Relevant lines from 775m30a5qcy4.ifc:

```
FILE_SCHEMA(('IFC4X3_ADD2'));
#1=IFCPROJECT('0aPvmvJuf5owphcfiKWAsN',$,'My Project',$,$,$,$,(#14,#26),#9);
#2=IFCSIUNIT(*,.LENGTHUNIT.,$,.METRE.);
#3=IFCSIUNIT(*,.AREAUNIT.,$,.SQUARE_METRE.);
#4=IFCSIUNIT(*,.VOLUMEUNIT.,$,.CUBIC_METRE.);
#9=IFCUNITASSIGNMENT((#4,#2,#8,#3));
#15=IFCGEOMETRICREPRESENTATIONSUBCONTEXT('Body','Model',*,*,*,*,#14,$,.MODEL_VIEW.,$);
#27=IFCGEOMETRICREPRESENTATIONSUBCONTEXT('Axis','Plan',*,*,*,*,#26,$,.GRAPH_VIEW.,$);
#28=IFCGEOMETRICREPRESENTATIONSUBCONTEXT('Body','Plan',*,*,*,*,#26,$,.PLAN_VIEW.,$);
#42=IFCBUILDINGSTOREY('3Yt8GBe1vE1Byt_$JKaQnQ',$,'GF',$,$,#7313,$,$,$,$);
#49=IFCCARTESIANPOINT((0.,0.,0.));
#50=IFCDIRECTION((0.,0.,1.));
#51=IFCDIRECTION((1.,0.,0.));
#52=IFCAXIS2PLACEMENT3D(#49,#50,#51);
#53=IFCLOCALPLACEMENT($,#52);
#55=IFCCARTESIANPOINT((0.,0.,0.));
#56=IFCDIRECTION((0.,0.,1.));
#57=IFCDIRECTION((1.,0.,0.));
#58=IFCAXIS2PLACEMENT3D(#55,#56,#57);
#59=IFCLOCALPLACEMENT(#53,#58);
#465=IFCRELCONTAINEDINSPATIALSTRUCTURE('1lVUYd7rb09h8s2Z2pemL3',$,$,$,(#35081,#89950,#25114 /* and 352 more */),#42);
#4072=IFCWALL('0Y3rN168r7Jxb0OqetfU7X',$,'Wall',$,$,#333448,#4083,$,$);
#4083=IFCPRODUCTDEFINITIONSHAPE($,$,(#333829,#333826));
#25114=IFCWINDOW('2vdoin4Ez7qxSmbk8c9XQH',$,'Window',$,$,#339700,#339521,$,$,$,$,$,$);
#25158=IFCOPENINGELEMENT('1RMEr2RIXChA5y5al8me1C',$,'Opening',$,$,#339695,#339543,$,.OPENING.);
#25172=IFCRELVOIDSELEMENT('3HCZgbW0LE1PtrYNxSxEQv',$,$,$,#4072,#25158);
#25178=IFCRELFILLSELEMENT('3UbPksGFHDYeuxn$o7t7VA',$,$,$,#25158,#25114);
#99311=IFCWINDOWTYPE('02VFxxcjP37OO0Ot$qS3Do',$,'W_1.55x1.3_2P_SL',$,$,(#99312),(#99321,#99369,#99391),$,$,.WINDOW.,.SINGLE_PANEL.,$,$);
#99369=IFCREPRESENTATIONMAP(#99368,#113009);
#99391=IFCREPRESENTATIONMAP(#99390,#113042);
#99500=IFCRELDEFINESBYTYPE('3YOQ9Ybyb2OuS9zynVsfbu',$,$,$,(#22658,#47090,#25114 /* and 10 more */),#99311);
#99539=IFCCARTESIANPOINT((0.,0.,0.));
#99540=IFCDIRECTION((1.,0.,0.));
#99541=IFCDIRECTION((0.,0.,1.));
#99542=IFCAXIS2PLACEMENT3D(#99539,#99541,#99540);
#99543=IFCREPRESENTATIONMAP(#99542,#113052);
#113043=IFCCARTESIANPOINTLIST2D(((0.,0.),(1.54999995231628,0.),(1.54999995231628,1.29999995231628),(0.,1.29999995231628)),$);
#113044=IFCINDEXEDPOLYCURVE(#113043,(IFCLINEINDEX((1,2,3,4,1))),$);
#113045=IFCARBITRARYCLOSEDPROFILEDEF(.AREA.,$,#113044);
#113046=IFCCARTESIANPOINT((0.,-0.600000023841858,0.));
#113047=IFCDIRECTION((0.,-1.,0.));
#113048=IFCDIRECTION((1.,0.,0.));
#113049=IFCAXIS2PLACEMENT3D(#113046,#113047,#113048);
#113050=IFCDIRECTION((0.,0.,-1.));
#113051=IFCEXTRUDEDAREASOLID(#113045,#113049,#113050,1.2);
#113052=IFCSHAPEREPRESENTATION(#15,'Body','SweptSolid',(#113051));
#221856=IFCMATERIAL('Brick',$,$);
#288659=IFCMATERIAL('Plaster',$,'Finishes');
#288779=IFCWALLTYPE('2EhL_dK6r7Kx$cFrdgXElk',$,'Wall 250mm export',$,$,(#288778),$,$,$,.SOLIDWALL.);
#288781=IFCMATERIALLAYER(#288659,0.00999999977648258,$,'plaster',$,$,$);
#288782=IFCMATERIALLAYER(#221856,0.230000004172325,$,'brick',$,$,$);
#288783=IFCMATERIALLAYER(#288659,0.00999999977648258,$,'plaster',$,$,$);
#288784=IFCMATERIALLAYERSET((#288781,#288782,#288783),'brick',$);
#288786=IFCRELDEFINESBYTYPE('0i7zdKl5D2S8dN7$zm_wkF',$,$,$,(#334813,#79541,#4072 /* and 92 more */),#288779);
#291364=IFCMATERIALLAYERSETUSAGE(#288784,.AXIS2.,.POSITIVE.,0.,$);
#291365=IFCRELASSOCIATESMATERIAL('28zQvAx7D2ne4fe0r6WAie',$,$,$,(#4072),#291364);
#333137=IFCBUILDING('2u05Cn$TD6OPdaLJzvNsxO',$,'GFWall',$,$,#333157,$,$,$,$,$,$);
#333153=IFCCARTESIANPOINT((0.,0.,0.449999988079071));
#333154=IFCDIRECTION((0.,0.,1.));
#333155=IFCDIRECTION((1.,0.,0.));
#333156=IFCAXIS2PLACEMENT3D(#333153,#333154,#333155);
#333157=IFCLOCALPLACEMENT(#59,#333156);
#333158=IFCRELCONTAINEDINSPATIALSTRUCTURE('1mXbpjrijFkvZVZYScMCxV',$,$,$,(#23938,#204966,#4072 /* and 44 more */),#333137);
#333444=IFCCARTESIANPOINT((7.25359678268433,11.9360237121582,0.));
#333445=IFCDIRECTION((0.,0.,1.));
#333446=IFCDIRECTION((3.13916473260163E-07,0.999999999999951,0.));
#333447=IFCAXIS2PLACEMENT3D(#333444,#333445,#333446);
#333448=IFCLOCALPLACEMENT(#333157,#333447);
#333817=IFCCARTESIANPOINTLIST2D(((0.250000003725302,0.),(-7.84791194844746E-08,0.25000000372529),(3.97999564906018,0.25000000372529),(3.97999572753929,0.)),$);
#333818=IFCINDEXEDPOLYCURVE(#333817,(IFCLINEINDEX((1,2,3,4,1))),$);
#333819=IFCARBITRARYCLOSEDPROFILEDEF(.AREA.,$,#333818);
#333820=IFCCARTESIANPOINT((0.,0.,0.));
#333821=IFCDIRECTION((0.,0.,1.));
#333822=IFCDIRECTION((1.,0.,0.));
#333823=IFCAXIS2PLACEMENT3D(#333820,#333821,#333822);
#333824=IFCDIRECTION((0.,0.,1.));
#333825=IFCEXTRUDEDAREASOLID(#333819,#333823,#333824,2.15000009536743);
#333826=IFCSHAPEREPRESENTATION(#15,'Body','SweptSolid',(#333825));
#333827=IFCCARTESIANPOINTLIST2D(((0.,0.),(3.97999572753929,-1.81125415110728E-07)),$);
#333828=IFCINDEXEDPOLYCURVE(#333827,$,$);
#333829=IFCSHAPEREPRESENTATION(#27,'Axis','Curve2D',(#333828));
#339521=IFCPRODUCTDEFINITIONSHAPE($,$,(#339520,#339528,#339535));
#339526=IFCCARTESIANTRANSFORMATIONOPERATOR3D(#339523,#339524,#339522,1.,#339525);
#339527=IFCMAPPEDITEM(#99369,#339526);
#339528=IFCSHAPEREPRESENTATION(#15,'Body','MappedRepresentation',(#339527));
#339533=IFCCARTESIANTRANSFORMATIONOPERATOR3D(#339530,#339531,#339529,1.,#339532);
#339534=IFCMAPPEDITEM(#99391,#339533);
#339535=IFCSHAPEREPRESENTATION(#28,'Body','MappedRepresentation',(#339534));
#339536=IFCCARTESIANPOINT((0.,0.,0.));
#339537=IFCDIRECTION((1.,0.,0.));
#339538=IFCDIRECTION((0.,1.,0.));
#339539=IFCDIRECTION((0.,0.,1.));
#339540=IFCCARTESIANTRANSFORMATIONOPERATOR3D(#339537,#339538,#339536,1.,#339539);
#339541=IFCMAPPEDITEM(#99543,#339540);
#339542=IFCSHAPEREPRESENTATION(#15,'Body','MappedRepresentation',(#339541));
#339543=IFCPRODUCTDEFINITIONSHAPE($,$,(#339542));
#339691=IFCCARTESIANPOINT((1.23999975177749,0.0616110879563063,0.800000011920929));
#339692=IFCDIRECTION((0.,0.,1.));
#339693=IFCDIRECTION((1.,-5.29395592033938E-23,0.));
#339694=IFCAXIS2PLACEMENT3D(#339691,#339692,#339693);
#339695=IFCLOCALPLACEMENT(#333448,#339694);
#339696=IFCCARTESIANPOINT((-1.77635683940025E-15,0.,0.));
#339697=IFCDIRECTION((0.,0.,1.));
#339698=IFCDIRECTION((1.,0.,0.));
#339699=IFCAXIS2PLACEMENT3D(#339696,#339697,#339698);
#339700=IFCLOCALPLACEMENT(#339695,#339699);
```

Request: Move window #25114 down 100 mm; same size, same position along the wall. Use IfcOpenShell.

```python
import numpy as np
import ifcopenshell
import ifcopenshell.api.geometry
import ifcopenshell.util.placement
import ifcopenshell.util.unit

model = ifcopenshell.open("775m30a5qcy4.ifc")
unit_scale = ifcopenshell.util.unit.calculate_unit_scale(model)

window = model.by_id(25114)
opening = window.FillsVoids[0].RelatingOpeningElement
dz = -0.1 / unit_scale

shift = np.array([0.0, 0.0, dz])
# The window is placed relative to its opening, so it follows when the opening moves.
matrix = ifcopenshell.util.placement.get_local_placement(opening.ObjectPlacement)
matrix[:3, 3] += shift
ifcopenshell.api.geometry.edit_object_placement(
    model, product=opening, matrix=matrix, is_si=False, should_transform_children=True
)

print(f"moved by {dz * unit_scale:+.3f} m")

model.write("775m30a5qcy4_edited.ifc")
```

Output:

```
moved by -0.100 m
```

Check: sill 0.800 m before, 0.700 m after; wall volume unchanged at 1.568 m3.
